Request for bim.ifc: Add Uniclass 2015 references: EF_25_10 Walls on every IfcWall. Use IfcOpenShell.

First a look at what the model holds.

```python
import ifcopenshell

model = ifcopenshell.open("bim.ifc")
print(model.schema)
print("classifications:", [c.Name for c in model.by_type("IfcClassification")])
for ifc_class in ("IfcDoor", "IfcRoof", "IfcStair", "IfcWall", "IfcWindow"):
    print(ifc_class, len(model.by_type(ifc_class)))
```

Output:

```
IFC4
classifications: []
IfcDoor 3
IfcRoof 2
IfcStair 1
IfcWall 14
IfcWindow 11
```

```python
import ifcopenshell
import ifcopenshell.api.classification

model = ifcopenshell.open("bim.ifc")

system = ifcopenshell.api.classification.add_classification(model, classification="Uniclass 2015")

codes = {
    "IfcWall": ("EF_25_10", "Walls"),
}
for ifc_class, (code, name) in codes.items():
    products = model.by_type(ifc_class)
    ifcopenshell.api.classification.add_reference(
        model, products=products, classification=system, identification=code, name=name
    )
    print(code, len(products))

model.write("bim_edited.ifc")
```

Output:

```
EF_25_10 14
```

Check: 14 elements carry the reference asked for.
